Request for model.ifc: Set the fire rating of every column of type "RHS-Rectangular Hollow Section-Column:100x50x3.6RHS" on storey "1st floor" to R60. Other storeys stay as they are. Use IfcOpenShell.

First a look at what the model holds.

```python
import ifcopenshell
import ifcopenshell.util.element

model = ifcopenshell.open("model.ifc")
print(model.schema)
storey = next(s for s in model.by_type("IfcBuildingStorey") if s.Name == "1st floor")
columns = [e for e in ifcopenshell.util.element.get_decomposition(storey) if e.is_a("IfcColumn")]
seen = {}
for e in columns:
    element_type = ifcopenshell.util.element.get_type(e)
    key = (element_type.Name if element_type != e and element_type else None, ifcopenshell.util.element.get_pset(e, "Pset_ColumnCommon", "FireRating"))
    seen[key] = seen.get(key, 0) + 1
for (name, value), count in sorted(seen.items(), key=str):
    print(count, "x", name, "|", value)
```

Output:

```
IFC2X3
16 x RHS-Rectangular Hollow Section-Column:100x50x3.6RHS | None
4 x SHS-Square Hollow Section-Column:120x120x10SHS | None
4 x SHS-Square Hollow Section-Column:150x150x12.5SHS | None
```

```python
import ifcopenshell
import ifcopenshell.api.pset
import ifcopenshell.util.element

model = ifcopenshell.open("model.ifc")

storey = next(s for s in model.by_type("IfcBuildingStorey") if s.Name == "1st floor")
columns = [e for e in ifcopenshell.util.element.get_decomposition(storey) if e.is_a("IfcColumn")]

count = 0
for e in columns:
    element_type = ifcopenshell.util.element.get_type(e)
    if element_type in (None, e) or element_type.Name != "RHS-Rectangular Hollow Section-Column:100x50x3.6RHS":
        continue
    # add_pset returns the element's existing set when there is one.
    pset = ifcopenshell.api.pset.add_pset(model, product=e, name="Pset_ColumnCommon")
    ifcopenshell.api.pset.edit_pset(model, pset=pset, properties={"FireRating": "R60"})
    count += 1

print(count, "columns updated")

model.write("model-out.ifc")
```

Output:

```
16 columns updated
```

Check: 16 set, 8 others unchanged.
